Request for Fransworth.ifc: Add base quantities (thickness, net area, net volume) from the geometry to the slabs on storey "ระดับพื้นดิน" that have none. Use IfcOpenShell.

First a look at what the model holds.

```python
import ifcopenshell
import ifcopenshell.util.element
import ifcopenshell.util.unit

model = ifcopenshell.open("Fransworth.ifc")
print(model.schema)
for unit_type in ("LENGTHUNIT", "AREAUNIT", "VOLUMEUNIT"):
    print(unit_type, ifcopenshell.util.unit.calculate_unit_scale(model, unit_type))
storey = next(s for s in model.by_type("IfcBuildingStorey") if s.Name == "ระดับพื้นดิน")
slabs = [e for e in ifcopenshell.util.element.get_decomposition(storey) if e.is_a("IfcSlab")]
for e in sorted(slabs, key=lambda e: e.id()):
    print(e.id(), e.is_a(), e.Name, list(ifcopenshell.util.element.get_psets(e, qtos_only=True)), sep=" | ")
```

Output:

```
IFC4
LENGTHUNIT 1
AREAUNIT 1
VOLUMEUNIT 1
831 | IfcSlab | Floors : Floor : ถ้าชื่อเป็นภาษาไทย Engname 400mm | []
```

```python
import ifcopenshell
import ifcopenshell.api.pset
import ifcopenshell.geom
import ifcopenshell.util.element
import ifcopenshell.util.shape
import ifcopenshell.util.unit

model = ifcopenshell.open("Fransworth.ifc")
unit_scale = ifcopenshell.util.unit.calculate_unit_scale(model)
area_scale = ifcopenshell.util.unit.calculate_unit_scale(model, "AREAUNIT")
volume_scale = ifcopenshell.util.unit.calculate_unit_scale(model, "VOLUMEUNIT")
settings = ifcopenshell.geom.settings()

storey = next(s for s in model.by_type("IfcBuildingStorey") if s.Name == "ระดับพื้นดิน")
slabs = [e for e in ifcopenshell.util.element.get_decomposition(storey) if e.is_a("IfcSlab")]

for e in sorted(slabs, key=lambda e: e.id()):
    if ifcopenshell.util.element.get_psets(e, qtos_only=True, should_inherit=False):
        continue
    # Geometry comes back in metres, in the element's own axes.
    shape = ifcopenshell.geom.create_shape(settings, e)
    values = {
        "Width": ifcopenshell.util.shape.get_z(shape.geometry) / unit_scale,
        "NetArea": ifcopenshell.util.shape.get_footprint_area(shape.geometry) / area_scale,
        "NetVolume": ifcopenshell.util.shape.get_volume(shape.geometry) / volume_scale,
    }
    qto = ifcopenshell.api.pset.add_qto(model, product=e, name="Qto_SlabBaseQuantities")
    ifcopenshell.api.pset.edit_qto(model, qto=qto, properties=values)
    print(e.id(), {k: round(v, 3) for k, v in values.items()})

model.write("Fransworth_updated.ifc")
```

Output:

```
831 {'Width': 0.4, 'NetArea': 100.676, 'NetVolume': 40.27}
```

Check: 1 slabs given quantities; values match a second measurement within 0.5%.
